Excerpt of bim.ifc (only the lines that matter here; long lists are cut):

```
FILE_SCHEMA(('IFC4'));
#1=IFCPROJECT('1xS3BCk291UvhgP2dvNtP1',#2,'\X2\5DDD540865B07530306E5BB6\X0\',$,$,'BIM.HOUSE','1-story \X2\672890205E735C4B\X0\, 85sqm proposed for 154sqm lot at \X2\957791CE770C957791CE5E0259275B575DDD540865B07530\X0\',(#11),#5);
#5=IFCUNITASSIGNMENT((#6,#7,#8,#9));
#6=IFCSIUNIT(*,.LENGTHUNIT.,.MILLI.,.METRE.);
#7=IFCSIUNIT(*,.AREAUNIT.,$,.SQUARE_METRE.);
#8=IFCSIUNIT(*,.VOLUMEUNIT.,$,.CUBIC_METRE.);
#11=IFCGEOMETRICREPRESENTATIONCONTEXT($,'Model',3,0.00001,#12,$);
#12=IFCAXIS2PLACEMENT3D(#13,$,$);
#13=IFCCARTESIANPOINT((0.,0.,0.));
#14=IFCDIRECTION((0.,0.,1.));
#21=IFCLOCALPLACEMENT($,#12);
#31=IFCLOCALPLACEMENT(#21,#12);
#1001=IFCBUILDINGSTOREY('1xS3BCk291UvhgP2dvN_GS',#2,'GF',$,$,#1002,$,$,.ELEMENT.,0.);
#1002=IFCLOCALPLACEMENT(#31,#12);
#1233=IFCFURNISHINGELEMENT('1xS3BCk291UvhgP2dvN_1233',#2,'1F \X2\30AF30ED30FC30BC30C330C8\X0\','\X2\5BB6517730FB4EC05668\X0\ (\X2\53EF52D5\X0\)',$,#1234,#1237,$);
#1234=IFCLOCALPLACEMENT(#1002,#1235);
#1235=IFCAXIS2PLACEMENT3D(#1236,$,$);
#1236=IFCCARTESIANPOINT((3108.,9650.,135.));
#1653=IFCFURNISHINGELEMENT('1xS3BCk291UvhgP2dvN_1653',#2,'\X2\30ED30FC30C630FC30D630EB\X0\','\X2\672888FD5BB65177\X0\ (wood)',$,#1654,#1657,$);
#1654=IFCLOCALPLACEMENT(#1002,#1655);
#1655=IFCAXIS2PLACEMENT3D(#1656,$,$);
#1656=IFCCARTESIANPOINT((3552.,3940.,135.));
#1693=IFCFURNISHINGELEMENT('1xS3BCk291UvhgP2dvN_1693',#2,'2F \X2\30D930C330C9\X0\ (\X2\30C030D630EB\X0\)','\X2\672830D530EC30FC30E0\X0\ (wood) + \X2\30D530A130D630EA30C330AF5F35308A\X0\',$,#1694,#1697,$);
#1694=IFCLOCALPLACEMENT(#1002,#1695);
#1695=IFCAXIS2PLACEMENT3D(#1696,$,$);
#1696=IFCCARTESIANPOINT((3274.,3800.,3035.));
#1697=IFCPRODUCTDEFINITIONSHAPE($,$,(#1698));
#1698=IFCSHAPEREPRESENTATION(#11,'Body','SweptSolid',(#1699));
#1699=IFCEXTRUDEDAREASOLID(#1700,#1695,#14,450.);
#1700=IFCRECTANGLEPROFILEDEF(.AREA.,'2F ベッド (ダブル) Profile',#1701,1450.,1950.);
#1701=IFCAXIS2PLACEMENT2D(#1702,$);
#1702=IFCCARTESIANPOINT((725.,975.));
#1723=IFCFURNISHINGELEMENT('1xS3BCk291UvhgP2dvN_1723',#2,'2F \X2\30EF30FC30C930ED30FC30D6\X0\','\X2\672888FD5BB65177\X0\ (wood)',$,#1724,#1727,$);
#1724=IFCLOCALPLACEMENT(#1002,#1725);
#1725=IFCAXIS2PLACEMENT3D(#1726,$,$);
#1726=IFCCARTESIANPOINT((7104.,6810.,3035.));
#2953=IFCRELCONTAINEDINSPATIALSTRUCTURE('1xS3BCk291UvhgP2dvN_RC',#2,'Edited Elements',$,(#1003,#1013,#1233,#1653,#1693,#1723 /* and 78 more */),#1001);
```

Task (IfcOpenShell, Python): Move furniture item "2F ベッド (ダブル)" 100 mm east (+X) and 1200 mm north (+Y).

```python
import ifcopenshell
import ifcopenshell.api.geometry
import ifcopenshell.util.placement
import ifcopenshell.util.unit

model = ifcopenshell.open("bim.ifc")
unit_scale = ifcopenshell.util.unit.calculate_unit_scale(model)

item = model.by_id(1693)
matrix = ifcopenshell.util.placement.get_local_placement(item.ObjectPlacement)
matrix[0, 3] += 0.1 / unit_scale
matrix[1, 3] += 1.2 / unit_scale
ifcopenshell.api.geometry.edit_object_placement(model, product=item, matrix=matrix, is_si=False)

print(ifcopenshell.util.placement.get_local_placement(item.ObjectPlacement).round(3) + 0.0)

model.write("bim_edited.ifc")
```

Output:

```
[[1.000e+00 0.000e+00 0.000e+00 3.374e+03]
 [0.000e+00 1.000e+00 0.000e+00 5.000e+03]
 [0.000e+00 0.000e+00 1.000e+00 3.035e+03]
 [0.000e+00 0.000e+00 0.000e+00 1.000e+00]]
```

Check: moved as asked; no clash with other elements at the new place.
